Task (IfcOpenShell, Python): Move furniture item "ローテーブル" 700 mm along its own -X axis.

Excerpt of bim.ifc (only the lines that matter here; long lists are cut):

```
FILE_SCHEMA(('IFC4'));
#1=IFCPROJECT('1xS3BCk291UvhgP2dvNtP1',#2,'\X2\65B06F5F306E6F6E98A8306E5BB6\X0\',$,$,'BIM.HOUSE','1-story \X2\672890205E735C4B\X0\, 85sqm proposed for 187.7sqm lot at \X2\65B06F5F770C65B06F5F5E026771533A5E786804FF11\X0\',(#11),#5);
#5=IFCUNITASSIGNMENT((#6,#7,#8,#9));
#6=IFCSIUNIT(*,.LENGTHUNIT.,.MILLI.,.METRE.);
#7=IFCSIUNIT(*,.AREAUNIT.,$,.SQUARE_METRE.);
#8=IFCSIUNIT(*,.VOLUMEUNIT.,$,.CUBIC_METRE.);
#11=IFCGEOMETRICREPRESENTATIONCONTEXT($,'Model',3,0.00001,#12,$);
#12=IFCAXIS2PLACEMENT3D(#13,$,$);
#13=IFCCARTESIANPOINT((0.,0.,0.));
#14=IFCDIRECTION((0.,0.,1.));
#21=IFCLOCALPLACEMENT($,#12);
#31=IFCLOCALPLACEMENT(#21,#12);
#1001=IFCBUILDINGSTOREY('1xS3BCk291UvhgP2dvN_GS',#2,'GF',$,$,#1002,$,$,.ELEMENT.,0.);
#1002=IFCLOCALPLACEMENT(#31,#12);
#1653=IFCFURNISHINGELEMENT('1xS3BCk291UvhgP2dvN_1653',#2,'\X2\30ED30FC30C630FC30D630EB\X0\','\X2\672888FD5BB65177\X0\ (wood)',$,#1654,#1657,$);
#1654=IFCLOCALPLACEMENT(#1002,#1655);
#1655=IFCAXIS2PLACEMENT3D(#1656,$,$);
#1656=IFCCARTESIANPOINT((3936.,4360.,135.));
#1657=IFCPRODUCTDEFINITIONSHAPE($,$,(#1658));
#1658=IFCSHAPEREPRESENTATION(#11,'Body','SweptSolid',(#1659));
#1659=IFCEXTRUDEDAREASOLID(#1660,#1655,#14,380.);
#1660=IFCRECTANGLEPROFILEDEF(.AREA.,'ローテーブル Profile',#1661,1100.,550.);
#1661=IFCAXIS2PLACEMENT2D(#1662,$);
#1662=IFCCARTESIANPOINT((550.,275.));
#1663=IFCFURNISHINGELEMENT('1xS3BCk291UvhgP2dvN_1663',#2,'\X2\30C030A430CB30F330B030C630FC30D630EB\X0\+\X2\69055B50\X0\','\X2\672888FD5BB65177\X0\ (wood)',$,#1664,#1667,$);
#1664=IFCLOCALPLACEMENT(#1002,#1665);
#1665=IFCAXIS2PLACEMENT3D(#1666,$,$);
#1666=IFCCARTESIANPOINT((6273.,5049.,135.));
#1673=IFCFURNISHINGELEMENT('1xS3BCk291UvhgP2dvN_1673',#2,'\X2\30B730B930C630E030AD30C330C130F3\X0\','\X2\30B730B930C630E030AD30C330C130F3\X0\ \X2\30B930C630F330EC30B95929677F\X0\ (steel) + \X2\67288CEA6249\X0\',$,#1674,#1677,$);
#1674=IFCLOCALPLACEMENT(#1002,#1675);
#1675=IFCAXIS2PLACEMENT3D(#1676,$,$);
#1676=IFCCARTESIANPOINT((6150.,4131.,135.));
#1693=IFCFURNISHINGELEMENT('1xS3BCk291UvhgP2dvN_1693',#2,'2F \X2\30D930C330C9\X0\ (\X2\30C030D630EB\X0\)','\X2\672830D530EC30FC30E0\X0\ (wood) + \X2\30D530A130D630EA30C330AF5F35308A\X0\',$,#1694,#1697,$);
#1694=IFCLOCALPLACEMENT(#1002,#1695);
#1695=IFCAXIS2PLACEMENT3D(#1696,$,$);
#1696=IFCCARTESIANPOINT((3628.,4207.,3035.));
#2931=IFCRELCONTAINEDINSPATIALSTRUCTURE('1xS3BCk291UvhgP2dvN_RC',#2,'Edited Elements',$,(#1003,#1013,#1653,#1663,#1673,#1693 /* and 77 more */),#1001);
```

```python
import ifcopenshell
import ifcopenshell.api.geometry
import ifcopenshell.util.placement

model = ifcopenshell.open("bim.ifc")

item = model.by_guid("1xS3BCk291UvhgP2dvN_1653")
matrix = ifcopenshell.util.placement.get_local_placement(item.ObjectPlacement)
matrix[:3, 3] -= matrix[:3, 0] * 700.0
ifcopenshell.api.geometry.edit_object_placement(model, product=item, matrix=matrix, is_si=False)

print(ifcopenshell.util.placement.get_local_placement(item.ObjectPlacement).round(3) + 0.0)

model.write("bim_edited.ifc")
```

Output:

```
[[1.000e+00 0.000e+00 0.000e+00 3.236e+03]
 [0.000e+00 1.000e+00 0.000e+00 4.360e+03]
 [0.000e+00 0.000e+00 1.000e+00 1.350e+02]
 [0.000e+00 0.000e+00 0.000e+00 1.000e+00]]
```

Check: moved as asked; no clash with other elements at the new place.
